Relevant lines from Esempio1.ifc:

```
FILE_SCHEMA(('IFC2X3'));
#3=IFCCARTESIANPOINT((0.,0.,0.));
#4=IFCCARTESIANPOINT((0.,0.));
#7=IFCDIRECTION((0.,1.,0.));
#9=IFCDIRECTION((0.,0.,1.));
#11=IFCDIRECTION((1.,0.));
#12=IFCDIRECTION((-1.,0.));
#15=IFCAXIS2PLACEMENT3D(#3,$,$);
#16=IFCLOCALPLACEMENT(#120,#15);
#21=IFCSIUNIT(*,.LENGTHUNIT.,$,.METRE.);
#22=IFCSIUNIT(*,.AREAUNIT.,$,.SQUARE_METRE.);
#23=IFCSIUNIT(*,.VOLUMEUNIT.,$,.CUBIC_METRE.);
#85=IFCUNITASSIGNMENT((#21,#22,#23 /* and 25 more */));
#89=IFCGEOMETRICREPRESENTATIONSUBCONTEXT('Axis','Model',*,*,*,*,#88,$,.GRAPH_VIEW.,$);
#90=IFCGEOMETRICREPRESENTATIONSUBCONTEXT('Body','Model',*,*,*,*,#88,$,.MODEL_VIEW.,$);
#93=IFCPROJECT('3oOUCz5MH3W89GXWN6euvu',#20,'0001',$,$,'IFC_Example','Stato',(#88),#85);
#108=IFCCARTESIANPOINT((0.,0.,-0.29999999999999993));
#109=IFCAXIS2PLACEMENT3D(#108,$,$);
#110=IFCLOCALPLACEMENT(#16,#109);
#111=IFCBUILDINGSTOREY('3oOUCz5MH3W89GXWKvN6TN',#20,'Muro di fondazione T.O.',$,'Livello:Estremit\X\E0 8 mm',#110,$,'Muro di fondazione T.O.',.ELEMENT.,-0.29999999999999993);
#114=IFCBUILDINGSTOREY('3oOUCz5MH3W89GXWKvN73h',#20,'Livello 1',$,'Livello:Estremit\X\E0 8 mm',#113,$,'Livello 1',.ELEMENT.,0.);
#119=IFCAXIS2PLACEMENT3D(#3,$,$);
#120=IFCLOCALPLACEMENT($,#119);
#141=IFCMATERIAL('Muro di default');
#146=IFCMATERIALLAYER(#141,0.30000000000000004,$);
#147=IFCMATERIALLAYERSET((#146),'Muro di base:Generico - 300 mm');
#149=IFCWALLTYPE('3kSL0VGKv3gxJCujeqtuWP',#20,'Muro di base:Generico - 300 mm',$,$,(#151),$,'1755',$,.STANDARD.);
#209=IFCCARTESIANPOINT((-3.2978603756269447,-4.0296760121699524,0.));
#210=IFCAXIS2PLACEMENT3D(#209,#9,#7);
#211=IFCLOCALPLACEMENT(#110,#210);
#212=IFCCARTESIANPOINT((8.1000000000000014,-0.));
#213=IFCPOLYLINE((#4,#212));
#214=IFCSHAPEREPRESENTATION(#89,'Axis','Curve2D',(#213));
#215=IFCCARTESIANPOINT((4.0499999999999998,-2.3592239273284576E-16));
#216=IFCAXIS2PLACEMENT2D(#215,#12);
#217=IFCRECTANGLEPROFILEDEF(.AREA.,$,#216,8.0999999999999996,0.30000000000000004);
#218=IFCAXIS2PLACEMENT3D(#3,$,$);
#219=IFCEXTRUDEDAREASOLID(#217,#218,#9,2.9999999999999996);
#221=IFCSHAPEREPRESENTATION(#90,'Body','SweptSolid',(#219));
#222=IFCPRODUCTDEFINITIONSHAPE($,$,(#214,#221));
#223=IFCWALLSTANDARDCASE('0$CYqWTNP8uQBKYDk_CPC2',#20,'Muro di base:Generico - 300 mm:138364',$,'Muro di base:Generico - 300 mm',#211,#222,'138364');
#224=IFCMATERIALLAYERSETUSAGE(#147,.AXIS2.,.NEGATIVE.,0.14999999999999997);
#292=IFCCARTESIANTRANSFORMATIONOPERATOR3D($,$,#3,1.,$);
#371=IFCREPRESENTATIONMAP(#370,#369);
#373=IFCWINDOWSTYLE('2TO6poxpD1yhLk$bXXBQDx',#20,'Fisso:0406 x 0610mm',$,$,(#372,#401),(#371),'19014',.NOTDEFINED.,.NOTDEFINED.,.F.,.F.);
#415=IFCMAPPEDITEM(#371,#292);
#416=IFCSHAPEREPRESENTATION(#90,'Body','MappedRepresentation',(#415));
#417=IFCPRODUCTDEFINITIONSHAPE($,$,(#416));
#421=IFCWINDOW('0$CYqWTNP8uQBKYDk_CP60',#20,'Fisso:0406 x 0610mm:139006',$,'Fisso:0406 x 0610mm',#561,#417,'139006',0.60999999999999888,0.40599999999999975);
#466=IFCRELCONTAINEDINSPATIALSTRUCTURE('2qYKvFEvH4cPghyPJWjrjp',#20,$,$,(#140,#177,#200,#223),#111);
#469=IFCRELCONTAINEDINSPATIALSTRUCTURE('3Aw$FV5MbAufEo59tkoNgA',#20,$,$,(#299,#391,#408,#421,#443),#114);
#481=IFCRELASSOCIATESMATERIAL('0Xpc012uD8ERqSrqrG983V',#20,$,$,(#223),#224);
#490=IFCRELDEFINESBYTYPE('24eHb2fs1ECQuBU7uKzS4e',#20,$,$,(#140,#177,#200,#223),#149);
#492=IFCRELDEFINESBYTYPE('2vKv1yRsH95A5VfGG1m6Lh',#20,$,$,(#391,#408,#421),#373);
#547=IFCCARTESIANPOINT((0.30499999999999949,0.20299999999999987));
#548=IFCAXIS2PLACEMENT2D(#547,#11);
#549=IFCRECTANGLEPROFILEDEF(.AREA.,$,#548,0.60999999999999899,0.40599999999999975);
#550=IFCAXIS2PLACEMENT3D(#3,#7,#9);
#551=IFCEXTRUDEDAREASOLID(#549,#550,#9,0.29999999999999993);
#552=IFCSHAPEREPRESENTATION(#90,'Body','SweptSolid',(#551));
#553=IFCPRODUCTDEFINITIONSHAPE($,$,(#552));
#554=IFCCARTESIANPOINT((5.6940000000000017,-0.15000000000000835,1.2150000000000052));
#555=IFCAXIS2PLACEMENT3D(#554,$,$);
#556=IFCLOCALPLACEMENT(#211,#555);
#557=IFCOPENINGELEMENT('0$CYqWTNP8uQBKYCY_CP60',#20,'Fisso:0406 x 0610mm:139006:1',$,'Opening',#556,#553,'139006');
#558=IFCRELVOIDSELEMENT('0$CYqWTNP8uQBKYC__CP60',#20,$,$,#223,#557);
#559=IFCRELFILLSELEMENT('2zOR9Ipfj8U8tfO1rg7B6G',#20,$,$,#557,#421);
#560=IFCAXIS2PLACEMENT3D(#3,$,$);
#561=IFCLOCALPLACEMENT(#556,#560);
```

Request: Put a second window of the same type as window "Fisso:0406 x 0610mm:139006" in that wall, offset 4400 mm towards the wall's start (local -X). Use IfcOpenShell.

```python
import ifcopenshell
import ifcopenshell.api.feature
import ifcopenshell.api.geometry
import ifcopenshell.api.root
import ifcopenshell.geom
import ifcopenshell.util.element
import ifcopenshell.util.placement
import ifcopenshell.util.shape
import ifcopenshell.util.unit

model = ifcopenshell.open("Esempio1.ifc")
unit_scale = ifcopenshell.util.unit.calculate_unit_scale(model)
settings = ifcopenshell.geom.settings()


def volume(element):
    """Net volume in cubic metres, openings subtracted."""
    shape = ifcopenshell.geom.create_shape(settings, element)
    return ifcopenshell.util.shape.get_volume(shape.geometry)


def reuse_history(source, copy):
    """copy_class also copies each property set's owner history, people and application; keep the originals."""
    for rel in copy.IsDefinedBy:
        if rel.is_a("IfcRelDefinesByProperties") and (history := rel.RelatingPropertyDefinition.OwnerHistory):
            rel.RelatingPropertyDefinition.OwnerHistory = source.OwnerHistory
            ifcopenshell.util.element.remove_deep2(model, history)


window = model.by_guid("0$CYqWTNP8uQBKYDk_CP60")
opening = window.FillsVoids[0].RelatingOpeningElement
wall = opening.VoidsElements[0].RelatingBuildingElement
before = volume(wall)
shift = ifcopenshell.util.placement.get_local_placement(wall.ObjectPlacement)[:3, 0] * -4.4 / unit_scale

# copy_class copies the void relationship, type, container and properties, but no geometry.
new_opening = ifcopenshell.api.root.copy_class(model, product=opening)
new_opening.Representation = ifcopenshell.util.element.copy_deep(
    model, opening.Representation, exclude=["IfcGeometricRepresentationContext", "IfcRepresentationMap"]
)
new_opening.Name = "Fisso:0406 x 0610mm"
new_opening.Tag = None
new_window = ifcopenshell.api.root.copy_class(model, product=window)
new_window.Representation = ifcopenshell.util.element.copy_deep(
    model, window.Representation, exclude=["IfcGeometricRepresentationContext", "IfcRepresentationMap"]
)
new_window.Name = "Fisso:0406 x 0610mm"
new_window.Tag = None
reuse_history(window, new_window)
fills = ifcopenshell.api.feature.add_filling(model, opening=new_opening, element=new_window)
fills.OwnerHistory = new_window.OwnerHistory  # required in IFC2X3

for old, new in ((opening, new_opening), (window, new_window)):
    matrix = ifcopenshell.util.placement.get_local_placement(old.ObjectPlacement)
    matrix[:3, 3] += shift
    ifcopenshell.api.geometry.edit_object_placement(model, product=new, matrix=matrix, is_si=False)

after = volume(wall)

print(f"wall volume {before:.3f} -> {after:.3f} m3")

model.write("Esempio1-out.ifc")
```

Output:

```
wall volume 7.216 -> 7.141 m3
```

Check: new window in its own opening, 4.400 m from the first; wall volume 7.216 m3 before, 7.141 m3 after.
